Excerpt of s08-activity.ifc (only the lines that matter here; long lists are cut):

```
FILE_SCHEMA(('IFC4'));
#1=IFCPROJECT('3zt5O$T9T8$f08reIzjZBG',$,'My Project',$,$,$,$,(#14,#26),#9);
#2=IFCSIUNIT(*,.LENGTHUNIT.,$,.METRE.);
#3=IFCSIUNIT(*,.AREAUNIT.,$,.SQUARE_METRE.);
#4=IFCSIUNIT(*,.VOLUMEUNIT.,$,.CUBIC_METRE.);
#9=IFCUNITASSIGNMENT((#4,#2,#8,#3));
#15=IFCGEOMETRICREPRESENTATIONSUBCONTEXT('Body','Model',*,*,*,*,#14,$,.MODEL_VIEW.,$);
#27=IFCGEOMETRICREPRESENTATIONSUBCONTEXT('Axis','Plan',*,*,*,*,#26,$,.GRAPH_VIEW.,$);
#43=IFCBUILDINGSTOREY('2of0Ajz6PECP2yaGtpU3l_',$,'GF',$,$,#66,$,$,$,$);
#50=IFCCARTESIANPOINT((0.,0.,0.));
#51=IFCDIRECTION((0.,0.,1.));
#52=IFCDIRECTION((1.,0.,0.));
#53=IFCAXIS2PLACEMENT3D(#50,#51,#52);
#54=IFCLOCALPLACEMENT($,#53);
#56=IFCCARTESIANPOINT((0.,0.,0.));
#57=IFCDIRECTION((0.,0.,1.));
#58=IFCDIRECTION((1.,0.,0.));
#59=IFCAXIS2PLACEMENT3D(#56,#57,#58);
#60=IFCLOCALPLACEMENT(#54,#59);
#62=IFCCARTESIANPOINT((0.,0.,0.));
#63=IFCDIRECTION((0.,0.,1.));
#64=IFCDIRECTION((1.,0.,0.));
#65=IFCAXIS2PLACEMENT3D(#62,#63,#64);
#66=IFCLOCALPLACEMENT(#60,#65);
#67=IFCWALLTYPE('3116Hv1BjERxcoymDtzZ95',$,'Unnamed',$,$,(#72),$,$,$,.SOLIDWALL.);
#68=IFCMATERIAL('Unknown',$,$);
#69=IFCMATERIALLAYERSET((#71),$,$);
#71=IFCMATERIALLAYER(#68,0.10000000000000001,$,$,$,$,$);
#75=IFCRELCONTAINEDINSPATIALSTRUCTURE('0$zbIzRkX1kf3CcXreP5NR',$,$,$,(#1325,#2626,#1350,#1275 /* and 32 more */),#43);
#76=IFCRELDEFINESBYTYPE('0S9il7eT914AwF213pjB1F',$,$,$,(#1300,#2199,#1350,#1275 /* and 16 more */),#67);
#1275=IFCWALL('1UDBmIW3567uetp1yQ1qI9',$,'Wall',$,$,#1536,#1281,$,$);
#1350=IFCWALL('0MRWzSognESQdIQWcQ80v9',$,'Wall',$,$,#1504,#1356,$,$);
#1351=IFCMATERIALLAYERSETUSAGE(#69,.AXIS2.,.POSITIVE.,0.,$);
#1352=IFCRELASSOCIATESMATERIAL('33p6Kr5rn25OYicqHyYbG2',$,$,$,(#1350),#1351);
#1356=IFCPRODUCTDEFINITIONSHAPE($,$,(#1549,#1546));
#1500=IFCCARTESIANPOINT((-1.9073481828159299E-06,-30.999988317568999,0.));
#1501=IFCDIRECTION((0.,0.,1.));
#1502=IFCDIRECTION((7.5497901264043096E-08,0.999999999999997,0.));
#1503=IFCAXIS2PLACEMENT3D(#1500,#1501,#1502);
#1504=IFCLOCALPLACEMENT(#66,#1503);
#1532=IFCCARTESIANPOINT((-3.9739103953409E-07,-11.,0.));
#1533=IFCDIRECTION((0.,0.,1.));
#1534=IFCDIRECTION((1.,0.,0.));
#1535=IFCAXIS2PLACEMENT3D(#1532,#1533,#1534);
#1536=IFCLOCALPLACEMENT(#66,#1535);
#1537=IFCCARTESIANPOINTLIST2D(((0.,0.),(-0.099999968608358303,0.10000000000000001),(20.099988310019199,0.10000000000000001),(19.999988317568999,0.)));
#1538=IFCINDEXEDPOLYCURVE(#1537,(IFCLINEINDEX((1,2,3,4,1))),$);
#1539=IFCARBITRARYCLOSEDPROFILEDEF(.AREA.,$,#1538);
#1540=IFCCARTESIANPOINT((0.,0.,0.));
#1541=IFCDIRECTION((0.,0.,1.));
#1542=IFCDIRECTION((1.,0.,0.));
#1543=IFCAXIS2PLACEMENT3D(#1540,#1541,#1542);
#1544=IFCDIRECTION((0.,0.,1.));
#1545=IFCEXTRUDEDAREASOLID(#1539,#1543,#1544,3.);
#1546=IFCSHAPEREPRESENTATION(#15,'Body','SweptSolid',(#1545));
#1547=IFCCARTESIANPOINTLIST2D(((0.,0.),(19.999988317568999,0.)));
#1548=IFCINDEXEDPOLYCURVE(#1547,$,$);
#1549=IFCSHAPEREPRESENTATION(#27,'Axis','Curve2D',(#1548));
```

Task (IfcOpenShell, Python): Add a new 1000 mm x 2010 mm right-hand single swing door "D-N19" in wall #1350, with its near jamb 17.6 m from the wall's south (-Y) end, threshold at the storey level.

```python
import numpy as np
import ifcopenshell
import ifcopenshell.api.feature
import ifcopenshell.api.geometry
import ifcopenshell.api.root
import ifcopenshell.api.spatial
import ifcopenshell.geom
import ifcopenshell.util.element
import ifcopenshell.util.placement
import ifcopenshell.util.representation
import ifcopenshell.util.shape
import ifcopenshell.util.unit

model = ifcopenshell.open("s08-activity.ifc")
unit_scale = ifcopenshell.util.unit.calculate_unit_scale(model)
settings = ifcopenshell.geom.settings()


def volume(element):
    """Net volume in cubic metres, openings subtracted."""
    shape = ifcopenshell.geom.create_shape(settings, element)
    return ifcopenshell.util.shape.get_volume(shape.geometry)


wall = model.by_guid("0MRWzSognESQdIQWcQ80v9")
storey = ifcopenshell.util.element.get_container(wall, ifc_class="IfcBuildingStorey")
context = ifcopenshell.util.representation.get_context(model, "Model", "Body", "MODEL_VIEW")
before = volume(wall)

width, height, from_end, sill = 1, 2.01, 17.6, 0.0  # metres

# The wall runs along its own X axis, and the end named is its -X end.
wall_shape = ifcopenshell.geom.create_shape(settings, wall)
x, y, z = ifcopenshell.util.shape.get_vertices(wall_shape.geometry).T
start = x.min() + from_end
face, thickness = float(y.min()), float(y.max() - y.min())
wall_matrix = ifcopenshell.util.placement.get_local_placement(wall.ObjectPlacement)
level = ifcopenshell.util.placement.get_local_placement(storey.ObjectPlacement)[2, 3]


def in_wall(x, y):
    """Placement at x, y metres in the wall's axes, at sill height."""
    matrix = wall_matrix.copy()
    matrix[:, 3] = wall_matrix @ np.array([x / unit_scale, y / unit_scale, 0.0, 1.0])
    matrix[2, 3] = level + sill / unit_scale
    return matrix


# Opening: a box that overshoots both wall faces by 50 mm.
opening = ifcopenshell.api.root.create_entity(model, ifc_class="IfcOpeningElement", predefined_type="OPENING")
box = ifcopenshell.api.geometry.add_wall_representation(
    model, context=context, length=width, height=height, thickness=thickness + 0.1
)
ifcopenshell.api.geometry.assign_representation(model, product=opening, representation=box)
ifcopenshell.api.geometry.edit_object_placement(model, product=opening, matrix=in_wall(start, face - 0.05), is_si=False)
ifcopenshell.api.feature.add_feature(model, feature=opening, element=wall)

door = ifcopenshell.api.root.create_entity(model, ifc_class="IfcDoor", name="D-N19", predefined_type="DOOR")
door.OverallWidth, door.OverallHeight = width / unit_scale, height / unit_scale
door.OperationType = "SINGLE_SWING_RIGHT"
body = ifcopenshell.api.geometry.add_door_representation(
    model,
    context=context,
    overall_width=door.OverallWidth,
    overall_height=door.OverallHeight,
    operation_type="SINGLE_SWING_RIGHT",
    lining_properties={"LiningDepth": thickness / unit_scale, "ThresholdDepth": thickness / unit_scale},
)
ifcopenshell.api.geometry.assign_representation(model, product=door, representation=body)
ifcopenshell.api.spatial.assign_container(model, products=[door], relating_structure=storey)
ifcopenshell.api.feature.add_filling(model, opening=opening, element=door)

# The lining spans the wall, so the door starts at the wall face.
ifcopenshell.api.geometry.edit_object_placement(model, product=door, matrix=in_wall(start, face), is_si=False)

after = volume(wall)

print(f"wall volume {before:.3f} -> {after:.3f} m3")

model.write("s08-activity_edited.ifc")
```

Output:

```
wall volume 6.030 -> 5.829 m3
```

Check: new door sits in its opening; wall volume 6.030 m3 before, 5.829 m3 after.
